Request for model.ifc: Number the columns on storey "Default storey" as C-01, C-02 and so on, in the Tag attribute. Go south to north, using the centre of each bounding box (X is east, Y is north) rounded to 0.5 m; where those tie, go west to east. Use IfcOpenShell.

First a look at what the model holds.

```python
import ifcopenshell
import ifcopenshell.util.element
import ifcopenshell.util.placement

model = ifcopenshell.open("model.ifc")
print(model.schema)
storey = next(s for s in model.by_type("IfcBuildingStorey") if s.Name == "Default storey")
columns = [e for e in ifcopenshell.util.element.get_decomposition(storey) if e.is_a("IfcColumn")]
for e in sorted(columns, key=lambda e: e.id()):
    origin = ifcopenshell.util.placement.get_local_placement(e.ObjectPlacement)[:3, 3]
    print(e.id(), e.Tag, e.Name, origin.round(2) + 0.0, sep=" | ")
```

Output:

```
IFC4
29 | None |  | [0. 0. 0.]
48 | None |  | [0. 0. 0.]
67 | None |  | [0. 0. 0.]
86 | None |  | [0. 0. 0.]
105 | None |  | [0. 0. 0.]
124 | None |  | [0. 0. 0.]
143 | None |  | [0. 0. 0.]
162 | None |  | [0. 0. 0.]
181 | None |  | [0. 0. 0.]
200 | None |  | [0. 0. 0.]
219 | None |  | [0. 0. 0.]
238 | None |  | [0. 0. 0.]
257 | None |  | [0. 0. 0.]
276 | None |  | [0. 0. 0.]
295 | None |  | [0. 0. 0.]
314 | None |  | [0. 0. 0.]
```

```python
import ifcopenshell
import ifcopenshell.geom
import ifcopenshell.util.element
import ifcopenshell.util.shape

model = ifcopenshell.open("model.ifc")
settings = ifcopenshell.geom.settings()
settings.set("use-world-coords", True)


def centre(element):
    shape = ifcopenshell.geom.create_shape(settings, element)
    return ifcopenshell.util.shape.get_bbox_centroid(shape.geometry)


storey = next(s for s in model.by_type("IfcBuildingStorey") if s.Name == "Default storey")
columns = [e for e in ifcopenshell.util.element.get_decomposition(storey) if e.is_a("IfcColumn")]

# Insertion points can sit at a corner or the storey origin, so sort by the geometry (in metres).
centres = {e: centre(e) for e in columns}
columns.sort(key=lambda e: (round(centres[e][1] / 0.5), centres[e][0]))

for i, e in enumerate(columns, start=1):
    number = f"C-{i:02d}"
    e.Tag = number
    print(e.id(), number)

model.write("model_updated.ifc")
```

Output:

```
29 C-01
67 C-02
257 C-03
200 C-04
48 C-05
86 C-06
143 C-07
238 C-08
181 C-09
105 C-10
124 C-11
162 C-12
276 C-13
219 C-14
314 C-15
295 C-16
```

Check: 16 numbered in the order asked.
